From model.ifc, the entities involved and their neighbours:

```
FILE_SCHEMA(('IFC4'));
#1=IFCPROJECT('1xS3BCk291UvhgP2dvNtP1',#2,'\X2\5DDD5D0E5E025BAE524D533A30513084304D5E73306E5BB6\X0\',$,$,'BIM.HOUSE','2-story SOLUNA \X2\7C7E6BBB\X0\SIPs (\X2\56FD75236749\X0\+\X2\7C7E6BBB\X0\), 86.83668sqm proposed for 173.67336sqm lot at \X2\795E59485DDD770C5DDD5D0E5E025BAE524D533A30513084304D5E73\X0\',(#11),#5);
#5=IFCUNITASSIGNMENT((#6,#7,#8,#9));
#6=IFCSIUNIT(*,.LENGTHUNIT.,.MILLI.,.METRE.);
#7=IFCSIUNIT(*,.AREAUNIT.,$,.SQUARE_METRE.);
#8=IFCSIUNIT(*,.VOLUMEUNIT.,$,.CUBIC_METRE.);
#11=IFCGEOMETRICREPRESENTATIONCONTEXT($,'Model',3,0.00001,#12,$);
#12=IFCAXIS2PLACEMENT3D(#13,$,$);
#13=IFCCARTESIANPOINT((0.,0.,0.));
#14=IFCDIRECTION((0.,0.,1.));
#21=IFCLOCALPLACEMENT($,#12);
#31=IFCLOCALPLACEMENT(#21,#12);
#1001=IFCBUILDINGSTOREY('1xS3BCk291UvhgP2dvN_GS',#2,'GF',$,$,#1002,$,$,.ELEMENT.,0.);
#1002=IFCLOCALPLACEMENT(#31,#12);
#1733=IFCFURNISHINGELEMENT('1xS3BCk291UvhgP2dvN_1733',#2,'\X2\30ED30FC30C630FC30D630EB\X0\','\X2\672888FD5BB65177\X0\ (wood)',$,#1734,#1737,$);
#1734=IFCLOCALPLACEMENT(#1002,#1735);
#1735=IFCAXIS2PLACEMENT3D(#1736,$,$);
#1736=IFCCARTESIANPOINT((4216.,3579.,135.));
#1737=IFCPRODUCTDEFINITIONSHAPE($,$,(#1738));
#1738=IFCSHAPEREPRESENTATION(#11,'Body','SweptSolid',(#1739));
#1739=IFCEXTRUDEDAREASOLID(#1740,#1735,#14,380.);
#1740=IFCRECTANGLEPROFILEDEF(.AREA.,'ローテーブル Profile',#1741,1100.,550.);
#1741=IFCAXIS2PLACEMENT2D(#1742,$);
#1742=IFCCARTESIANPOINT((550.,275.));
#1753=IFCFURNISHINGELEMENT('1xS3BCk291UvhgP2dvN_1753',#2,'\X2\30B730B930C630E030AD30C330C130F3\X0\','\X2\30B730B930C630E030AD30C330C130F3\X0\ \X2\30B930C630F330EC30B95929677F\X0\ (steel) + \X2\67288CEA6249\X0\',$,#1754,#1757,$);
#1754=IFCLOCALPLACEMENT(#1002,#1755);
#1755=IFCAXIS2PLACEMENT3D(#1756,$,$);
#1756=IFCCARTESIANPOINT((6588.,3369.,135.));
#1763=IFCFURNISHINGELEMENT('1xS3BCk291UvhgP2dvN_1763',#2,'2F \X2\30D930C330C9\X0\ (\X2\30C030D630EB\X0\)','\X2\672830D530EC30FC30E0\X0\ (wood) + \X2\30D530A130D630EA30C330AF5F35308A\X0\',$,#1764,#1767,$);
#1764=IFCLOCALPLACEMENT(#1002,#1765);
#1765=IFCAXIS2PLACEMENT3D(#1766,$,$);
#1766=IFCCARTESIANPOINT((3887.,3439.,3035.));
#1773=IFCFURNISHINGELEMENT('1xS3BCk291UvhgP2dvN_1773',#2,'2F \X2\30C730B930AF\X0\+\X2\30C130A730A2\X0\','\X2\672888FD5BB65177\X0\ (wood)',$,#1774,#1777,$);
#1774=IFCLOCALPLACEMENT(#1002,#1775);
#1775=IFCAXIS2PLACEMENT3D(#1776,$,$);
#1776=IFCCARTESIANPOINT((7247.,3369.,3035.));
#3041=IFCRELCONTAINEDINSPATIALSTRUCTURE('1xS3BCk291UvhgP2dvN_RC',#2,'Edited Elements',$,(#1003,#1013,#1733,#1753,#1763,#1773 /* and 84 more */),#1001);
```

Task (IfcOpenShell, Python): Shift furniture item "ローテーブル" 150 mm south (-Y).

```python
import ifcopenshell
import ifcopenshell.api.geometry
import ifcopenshell.util.placement
import ifcopenshell.util.unit

model = ifcopenshell.open("model.ifc")
unit_scale = ifcopenshell.util.unit.calculate_unit_scale(model)

item = model.by_guid("1xS3BCk291UvhgP2dvN_1733")
matrix = ifcopenshell.util.placement.get_local_placement(item.ObjectPlacement)
matrix[1, 3] -= 0.15 / unit_scale
ifcopenshell.api.geometry.edit_object_placement(model, product=item, matrix=matrix, is_si=False)

print(ifcopenshell.util.placement.get_local_placement(item.ObjectPlacement).round(3) + 0.0)

model.write("model_rev.ifc")
```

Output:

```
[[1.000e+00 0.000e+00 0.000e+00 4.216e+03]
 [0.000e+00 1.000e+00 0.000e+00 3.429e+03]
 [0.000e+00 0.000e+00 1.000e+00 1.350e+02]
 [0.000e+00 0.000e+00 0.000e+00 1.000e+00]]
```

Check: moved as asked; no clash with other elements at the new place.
